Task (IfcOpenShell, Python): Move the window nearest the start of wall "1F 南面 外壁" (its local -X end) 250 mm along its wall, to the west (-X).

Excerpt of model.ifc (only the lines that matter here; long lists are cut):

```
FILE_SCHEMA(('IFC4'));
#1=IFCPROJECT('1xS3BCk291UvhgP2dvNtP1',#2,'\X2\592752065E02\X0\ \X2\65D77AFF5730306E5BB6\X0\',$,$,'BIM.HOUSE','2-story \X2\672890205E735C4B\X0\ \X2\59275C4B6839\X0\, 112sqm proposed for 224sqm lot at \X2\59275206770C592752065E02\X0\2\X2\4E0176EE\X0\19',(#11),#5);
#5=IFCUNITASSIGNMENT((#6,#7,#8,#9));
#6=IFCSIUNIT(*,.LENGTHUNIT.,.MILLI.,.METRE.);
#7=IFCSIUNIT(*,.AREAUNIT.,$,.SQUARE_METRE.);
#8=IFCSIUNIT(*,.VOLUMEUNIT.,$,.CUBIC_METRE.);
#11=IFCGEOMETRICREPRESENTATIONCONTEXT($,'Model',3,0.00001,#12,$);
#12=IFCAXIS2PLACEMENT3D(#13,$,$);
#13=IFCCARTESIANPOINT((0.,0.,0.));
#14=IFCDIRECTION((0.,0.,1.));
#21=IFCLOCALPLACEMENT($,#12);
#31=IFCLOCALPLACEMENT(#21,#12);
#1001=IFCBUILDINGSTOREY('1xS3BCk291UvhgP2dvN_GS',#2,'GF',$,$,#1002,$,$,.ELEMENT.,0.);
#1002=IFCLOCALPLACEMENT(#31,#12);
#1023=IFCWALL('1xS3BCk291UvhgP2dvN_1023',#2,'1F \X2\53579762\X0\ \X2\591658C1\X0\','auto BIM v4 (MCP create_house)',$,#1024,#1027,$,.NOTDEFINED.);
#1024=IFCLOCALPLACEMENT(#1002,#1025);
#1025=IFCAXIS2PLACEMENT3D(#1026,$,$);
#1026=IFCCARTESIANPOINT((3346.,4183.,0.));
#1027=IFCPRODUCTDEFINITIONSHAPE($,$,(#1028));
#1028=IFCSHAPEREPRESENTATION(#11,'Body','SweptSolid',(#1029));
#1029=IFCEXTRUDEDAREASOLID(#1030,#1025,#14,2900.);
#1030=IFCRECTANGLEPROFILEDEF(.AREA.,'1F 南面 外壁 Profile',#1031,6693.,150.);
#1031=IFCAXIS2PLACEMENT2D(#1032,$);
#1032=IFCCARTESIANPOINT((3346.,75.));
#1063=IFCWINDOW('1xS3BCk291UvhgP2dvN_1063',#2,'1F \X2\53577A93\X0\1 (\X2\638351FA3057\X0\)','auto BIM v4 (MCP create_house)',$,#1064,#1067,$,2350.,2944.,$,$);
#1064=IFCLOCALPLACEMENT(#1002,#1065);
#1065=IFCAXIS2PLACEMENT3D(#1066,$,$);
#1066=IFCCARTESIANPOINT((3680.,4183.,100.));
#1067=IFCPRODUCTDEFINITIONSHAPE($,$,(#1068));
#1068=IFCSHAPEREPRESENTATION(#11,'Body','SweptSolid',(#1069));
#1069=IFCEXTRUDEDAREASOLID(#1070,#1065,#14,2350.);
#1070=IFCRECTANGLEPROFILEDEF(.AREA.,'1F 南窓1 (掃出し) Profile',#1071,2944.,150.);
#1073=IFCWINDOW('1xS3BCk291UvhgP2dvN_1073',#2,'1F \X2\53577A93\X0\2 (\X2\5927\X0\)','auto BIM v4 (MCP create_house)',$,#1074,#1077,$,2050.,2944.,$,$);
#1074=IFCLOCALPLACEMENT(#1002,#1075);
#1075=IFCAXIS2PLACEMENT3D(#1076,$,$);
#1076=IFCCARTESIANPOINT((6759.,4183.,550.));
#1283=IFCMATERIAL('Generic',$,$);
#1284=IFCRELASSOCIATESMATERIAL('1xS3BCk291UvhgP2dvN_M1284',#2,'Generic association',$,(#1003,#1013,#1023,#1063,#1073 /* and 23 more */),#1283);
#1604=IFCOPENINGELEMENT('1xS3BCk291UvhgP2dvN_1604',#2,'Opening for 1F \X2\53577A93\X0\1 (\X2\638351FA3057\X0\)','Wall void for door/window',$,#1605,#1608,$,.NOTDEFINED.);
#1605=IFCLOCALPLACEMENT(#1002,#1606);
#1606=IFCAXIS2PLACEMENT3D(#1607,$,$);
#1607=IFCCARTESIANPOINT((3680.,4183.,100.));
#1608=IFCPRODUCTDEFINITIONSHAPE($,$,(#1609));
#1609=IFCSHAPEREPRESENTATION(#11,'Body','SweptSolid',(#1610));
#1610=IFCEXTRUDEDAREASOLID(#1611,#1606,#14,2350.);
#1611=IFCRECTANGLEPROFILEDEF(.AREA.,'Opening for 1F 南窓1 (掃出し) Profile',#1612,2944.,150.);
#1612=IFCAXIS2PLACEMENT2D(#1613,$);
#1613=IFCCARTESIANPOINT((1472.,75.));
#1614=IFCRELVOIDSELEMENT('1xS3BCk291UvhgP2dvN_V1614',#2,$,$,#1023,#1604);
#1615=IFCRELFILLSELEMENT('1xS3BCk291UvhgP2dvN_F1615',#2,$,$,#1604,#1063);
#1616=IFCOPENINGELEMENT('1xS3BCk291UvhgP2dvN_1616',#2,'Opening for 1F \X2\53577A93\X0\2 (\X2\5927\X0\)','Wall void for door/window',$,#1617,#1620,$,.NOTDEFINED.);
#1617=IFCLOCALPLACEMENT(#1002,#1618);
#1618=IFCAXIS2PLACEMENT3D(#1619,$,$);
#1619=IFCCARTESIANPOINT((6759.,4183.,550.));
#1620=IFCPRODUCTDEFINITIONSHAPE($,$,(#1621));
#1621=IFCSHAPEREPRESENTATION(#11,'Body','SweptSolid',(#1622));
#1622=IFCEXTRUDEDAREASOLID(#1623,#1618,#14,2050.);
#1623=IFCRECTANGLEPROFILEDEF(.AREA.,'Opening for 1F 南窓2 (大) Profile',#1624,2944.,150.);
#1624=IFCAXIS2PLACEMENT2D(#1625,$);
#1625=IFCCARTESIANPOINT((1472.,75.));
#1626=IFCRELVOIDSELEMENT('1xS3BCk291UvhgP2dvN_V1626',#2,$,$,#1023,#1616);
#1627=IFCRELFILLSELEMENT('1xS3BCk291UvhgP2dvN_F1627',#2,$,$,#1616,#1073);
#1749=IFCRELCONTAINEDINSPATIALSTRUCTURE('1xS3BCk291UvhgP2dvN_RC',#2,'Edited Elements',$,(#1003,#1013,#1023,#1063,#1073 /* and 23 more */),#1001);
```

```python
import ifcopenshell
import ifcopenshell.api.geometry
import ifcopenshell.util.placement
import ifcopenshell.util.unit

model = ifcopenshell.open("model.ifc")
unit_scale = ifcopenshell.util.unit.calculate_unit_scale(model)

window = model.by_guid("1xS3BCk291UvhgP2dvN_1063")
opening = window.FillsVoids[0].RelatingOpeningElement
wall = opening.VoidsElements[0].RelatingBuildingElement

wall_matrix = ifcopenshell.util.placement.get_local_placement(wall.ObjectPlacement)
shift = wall_matrix[:3, 0] * -0.25 / unit_scale
before = ifcopenshell.util.placement.get_local_placement(window.ObjectPlacement)[:3, 3].copy()

# The window is not placed relative to its opening, so move both.
for product in (opening, window):
    matrix = ifcopenshell.util.placement.get_local_placement(product.ObjectPlacement)
    matrix[:3, 3] += shift
    ifcopenshell.api.geometry.edit_object_placement(model, product=product, matrix=matrix, is_si=False)

after = ifcopenshell.util.placement.get_local_placement(window.ObjectPlacement)[:3, 3]
print("window moved by", (after - before).round(3) + 0.0)

model.write("model-out.ifc")
```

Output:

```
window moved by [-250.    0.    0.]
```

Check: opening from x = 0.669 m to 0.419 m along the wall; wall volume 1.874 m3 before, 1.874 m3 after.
